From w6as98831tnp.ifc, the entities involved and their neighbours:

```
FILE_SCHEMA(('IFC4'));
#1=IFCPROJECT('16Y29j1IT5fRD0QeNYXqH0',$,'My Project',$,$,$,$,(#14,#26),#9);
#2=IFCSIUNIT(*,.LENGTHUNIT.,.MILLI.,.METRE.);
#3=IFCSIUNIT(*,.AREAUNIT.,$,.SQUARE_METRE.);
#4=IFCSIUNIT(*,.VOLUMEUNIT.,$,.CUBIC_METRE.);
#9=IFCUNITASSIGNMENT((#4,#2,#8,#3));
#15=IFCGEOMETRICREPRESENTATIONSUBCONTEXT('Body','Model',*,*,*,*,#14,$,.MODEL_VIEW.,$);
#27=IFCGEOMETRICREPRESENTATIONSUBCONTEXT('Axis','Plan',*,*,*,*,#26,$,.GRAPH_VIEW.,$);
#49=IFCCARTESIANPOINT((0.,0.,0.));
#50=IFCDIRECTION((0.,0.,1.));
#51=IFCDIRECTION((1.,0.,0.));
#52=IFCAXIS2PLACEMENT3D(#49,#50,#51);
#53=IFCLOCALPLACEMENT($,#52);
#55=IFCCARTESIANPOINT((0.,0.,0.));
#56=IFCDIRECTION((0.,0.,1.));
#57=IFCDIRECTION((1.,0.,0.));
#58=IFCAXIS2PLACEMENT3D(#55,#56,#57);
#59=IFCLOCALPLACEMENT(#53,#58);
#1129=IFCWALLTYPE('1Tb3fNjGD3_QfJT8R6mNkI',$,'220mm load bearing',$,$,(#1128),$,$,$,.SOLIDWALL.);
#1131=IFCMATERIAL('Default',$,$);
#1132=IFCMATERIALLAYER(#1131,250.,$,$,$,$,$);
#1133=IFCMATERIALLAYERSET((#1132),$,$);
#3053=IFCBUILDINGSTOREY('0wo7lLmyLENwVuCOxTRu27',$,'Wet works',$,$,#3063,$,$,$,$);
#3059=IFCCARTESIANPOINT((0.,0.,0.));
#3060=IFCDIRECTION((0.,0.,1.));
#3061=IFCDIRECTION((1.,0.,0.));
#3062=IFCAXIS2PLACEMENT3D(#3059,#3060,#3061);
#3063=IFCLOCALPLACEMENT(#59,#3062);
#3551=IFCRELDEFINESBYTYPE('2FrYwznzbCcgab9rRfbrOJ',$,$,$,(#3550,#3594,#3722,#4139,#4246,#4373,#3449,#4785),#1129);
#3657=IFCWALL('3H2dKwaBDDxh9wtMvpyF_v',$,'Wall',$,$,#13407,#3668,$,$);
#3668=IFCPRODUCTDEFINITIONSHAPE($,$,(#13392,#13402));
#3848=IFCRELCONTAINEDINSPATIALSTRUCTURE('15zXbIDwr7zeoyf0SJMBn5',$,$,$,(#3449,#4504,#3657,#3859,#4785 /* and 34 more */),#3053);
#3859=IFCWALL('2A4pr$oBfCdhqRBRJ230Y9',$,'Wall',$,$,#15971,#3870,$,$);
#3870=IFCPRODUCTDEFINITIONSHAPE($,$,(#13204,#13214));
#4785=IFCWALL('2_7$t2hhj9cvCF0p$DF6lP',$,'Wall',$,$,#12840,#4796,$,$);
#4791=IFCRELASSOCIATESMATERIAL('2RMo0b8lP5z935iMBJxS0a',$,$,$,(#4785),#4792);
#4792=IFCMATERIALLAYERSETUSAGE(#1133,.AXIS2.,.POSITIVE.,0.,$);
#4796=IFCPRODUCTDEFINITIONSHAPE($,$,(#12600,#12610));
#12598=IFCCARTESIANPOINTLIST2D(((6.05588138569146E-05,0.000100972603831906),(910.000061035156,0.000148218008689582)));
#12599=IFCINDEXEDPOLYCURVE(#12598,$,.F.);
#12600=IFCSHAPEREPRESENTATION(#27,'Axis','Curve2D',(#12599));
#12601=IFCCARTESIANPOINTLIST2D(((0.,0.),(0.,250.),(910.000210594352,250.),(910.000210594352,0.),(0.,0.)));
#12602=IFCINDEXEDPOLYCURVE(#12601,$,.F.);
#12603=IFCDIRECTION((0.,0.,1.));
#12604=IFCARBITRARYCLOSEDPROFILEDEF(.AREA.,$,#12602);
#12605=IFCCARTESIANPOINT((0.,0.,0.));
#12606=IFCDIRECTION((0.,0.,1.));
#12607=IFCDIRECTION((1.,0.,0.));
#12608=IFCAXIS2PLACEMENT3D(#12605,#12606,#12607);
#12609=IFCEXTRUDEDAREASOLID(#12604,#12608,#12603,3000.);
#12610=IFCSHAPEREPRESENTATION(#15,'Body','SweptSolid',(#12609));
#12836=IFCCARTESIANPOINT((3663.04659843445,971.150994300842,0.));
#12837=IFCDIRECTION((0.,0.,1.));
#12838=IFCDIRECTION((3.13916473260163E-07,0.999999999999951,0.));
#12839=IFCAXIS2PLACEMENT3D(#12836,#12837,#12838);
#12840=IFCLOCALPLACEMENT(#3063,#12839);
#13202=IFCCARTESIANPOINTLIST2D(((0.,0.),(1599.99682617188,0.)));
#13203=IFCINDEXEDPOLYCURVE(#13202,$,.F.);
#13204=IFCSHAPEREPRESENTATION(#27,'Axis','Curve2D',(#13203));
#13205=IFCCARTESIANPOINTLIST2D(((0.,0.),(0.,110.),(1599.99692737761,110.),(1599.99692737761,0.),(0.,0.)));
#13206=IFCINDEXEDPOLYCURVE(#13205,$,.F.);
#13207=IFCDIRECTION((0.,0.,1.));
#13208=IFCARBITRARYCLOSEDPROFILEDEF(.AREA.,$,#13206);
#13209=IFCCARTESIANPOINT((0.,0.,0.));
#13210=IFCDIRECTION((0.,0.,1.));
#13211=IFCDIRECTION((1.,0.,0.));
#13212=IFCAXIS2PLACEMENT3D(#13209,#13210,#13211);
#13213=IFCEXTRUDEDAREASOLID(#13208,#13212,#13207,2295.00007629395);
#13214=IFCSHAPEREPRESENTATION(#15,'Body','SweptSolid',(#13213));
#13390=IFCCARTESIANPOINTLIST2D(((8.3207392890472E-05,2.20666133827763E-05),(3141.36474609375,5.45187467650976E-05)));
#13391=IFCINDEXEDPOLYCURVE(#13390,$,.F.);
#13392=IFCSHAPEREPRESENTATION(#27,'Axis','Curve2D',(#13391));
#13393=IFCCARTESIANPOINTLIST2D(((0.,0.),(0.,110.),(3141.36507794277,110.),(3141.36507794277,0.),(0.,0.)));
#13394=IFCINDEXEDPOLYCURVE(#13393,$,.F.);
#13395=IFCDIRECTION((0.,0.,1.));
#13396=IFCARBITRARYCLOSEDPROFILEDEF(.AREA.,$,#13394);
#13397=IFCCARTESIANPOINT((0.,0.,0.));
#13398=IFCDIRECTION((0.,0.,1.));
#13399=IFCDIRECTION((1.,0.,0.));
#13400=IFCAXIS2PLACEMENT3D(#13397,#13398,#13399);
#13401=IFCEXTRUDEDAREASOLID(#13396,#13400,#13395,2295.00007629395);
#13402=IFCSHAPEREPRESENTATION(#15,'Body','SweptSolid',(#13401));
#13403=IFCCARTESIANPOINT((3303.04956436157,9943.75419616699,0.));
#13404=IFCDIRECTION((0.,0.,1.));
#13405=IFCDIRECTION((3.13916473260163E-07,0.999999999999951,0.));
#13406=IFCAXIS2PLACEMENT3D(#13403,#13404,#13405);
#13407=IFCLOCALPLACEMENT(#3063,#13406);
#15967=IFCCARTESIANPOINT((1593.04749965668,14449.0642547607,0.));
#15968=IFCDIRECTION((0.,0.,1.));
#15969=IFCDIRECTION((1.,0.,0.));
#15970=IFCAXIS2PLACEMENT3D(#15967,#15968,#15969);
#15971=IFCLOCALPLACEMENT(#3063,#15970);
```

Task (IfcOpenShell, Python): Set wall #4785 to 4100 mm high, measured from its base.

```python
import ifcopenshell
import ifcopenshell.geom
import ifcopenshell.util.representation
import ifcopenshell.util.shape
import ifcopenshell.util.unit

model = ifcopenshell.open("w6as98831tnp.ifc")
unit_scale = ifcopenshell.util.unit.calculate_unit_scale(model)
settings = ifcopenshell.geom.settings()


def volume(element):
    """Net volume in cubic metres, openings subtracted."""
    shape = ifcopenshell.geom.create_shape(settings, element)
    return ifcopenshell.util.shape.get_volume(shape.geometry)


wall = model.by_guid("2_7$t2hhj9cvCF0p$DF6lP")
before = volume(wall)

body = ifcopenshell.util.representation.get_representation(wall, "Model", "Body")
solid = body.Items[0]
old_height = solid.Depth
solid.Depth = 4.1 / unit_scale
after = volume(wall)

print(f"height {old_height:g} -> {solid.Depth:g}, volume {before:.3f} -> {after:.3f} m3")

model.write("w6as98831tnp_rev.ifc")
```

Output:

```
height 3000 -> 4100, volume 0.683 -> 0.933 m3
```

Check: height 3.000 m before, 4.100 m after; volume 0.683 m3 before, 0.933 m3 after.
